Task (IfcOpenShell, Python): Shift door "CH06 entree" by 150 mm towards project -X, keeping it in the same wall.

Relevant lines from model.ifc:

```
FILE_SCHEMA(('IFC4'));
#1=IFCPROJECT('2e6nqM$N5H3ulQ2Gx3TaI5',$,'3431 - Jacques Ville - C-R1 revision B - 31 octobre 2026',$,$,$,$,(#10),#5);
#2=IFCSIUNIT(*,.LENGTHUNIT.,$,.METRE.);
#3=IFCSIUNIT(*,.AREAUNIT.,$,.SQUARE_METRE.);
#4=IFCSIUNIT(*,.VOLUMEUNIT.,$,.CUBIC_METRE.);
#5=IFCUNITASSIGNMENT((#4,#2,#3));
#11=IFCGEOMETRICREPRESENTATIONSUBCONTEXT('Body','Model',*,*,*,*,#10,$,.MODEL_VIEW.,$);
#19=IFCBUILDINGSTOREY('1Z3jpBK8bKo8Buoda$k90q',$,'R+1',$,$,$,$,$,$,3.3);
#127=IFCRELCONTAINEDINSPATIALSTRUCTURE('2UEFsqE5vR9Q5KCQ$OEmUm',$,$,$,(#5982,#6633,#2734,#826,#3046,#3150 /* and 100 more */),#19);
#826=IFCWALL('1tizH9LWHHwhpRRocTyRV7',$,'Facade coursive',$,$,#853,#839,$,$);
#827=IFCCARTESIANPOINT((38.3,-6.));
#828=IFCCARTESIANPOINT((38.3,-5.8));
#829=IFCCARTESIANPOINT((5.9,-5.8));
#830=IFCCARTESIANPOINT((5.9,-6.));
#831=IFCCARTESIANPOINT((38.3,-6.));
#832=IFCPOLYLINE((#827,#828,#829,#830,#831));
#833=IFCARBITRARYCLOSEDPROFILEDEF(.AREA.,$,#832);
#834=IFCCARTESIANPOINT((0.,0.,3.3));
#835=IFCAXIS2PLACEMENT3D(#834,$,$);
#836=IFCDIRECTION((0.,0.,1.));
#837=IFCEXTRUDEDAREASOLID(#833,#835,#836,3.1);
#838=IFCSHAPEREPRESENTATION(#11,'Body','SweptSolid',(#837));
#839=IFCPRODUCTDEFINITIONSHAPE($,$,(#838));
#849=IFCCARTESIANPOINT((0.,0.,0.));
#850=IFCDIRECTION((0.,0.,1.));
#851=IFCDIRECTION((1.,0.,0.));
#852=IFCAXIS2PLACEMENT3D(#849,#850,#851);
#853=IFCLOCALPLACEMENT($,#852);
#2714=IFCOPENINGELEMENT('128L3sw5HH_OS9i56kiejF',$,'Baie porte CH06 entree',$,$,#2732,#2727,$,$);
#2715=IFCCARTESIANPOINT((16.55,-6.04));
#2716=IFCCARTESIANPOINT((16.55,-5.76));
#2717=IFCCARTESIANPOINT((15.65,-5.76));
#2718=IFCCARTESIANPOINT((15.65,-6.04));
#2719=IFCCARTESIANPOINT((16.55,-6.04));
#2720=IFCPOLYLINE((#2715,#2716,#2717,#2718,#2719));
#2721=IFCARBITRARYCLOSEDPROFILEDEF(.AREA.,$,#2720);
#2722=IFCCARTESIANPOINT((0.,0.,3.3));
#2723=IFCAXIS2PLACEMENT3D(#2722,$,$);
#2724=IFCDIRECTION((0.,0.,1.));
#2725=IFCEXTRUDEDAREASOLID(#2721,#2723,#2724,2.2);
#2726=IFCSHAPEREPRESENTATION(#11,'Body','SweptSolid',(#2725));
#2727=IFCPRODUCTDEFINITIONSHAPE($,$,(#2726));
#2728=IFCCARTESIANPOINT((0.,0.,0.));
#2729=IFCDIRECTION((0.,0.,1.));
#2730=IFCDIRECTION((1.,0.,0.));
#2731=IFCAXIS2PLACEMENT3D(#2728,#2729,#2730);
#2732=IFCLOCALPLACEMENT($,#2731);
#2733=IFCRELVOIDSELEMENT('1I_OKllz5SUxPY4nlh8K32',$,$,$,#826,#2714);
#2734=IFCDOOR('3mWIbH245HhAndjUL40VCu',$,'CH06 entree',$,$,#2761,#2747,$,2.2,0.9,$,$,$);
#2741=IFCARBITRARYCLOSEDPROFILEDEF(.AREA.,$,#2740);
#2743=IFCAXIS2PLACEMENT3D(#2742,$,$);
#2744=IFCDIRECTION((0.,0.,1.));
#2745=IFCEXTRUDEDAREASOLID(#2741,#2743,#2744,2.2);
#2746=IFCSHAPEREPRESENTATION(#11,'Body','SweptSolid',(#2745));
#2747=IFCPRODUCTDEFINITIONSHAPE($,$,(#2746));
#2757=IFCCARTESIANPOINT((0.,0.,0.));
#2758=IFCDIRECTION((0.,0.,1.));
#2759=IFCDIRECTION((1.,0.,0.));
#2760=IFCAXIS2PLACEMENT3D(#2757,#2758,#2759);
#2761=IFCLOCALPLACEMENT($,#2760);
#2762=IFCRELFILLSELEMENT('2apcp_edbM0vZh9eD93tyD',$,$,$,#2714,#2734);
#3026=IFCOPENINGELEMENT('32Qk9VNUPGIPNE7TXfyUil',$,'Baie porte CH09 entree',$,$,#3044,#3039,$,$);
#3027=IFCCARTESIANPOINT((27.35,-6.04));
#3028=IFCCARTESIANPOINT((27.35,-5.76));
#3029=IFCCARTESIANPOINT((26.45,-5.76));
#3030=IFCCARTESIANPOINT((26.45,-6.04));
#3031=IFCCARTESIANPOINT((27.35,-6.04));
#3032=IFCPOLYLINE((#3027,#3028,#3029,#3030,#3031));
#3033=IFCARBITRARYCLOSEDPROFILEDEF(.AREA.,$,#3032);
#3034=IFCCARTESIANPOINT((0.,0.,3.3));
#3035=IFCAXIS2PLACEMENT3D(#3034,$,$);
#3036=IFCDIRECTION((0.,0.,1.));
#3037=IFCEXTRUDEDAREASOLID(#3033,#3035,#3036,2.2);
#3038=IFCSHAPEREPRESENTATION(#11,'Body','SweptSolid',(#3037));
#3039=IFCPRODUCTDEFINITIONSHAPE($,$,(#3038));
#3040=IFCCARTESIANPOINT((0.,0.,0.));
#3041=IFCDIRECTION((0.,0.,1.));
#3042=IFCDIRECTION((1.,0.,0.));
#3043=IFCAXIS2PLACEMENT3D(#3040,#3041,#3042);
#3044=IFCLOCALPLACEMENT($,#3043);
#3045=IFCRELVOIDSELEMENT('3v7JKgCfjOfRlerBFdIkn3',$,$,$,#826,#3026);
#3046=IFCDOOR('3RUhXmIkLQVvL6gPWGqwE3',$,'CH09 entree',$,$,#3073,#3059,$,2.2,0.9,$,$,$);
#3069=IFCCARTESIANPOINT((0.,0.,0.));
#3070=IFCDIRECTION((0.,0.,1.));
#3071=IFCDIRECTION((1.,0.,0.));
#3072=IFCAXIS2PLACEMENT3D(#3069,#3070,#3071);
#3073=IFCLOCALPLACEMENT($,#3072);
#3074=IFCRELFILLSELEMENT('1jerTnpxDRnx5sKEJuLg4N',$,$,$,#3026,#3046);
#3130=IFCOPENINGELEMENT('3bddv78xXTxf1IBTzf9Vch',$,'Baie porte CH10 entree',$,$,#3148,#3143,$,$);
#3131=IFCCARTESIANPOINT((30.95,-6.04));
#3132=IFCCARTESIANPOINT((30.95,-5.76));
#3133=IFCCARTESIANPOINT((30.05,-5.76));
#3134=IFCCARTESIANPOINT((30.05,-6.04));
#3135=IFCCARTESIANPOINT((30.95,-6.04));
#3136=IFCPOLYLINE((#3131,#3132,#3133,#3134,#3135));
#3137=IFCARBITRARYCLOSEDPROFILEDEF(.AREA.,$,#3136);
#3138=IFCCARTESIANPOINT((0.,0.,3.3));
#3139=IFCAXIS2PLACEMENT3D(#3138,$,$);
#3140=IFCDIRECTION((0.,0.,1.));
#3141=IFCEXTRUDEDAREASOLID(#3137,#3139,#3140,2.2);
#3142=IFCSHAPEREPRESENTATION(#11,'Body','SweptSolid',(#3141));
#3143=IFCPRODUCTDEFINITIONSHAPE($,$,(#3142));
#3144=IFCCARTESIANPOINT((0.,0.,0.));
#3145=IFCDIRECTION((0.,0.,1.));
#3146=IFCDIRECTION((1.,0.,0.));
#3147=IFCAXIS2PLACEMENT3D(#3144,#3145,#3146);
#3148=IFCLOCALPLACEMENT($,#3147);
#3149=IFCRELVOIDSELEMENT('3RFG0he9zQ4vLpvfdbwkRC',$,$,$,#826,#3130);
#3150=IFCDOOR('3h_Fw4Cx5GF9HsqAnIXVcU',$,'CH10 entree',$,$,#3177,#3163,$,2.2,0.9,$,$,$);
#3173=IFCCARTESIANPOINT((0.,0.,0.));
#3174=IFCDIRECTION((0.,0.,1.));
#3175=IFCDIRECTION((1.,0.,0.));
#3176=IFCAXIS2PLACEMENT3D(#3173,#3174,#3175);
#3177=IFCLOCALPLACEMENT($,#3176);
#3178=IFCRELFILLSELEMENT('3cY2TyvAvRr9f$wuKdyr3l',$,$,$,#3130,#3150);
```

```python
import ifcopenshell
import ifcopenshell.api.geometry
import ifcopenshell.util.placement
import ifcopenshell.util.unit

model = ifcopenshell.open("model.ifc")
unit_scale = ifcopenshell.util.unit.calculate_unit_scale(model)

door = model.by_guid("3mWIbH245HhAndjUL40VCu")
opening = door.FillsVoids[0].RelatingOpeningElement
wall = opening.VoidsElements[0].RelatingBuildingElement

wall_matrix = ifcopenshell.util.placement.get_local_placement(wall.ObjectPlacement)
shift = wall_matrix[:3, 0] * -0.15 / unit_scale
before = ifcopenshell.util.placement.get_local_placement(door.ObjectPlacement)[:3, 3].copy()

# The door is not placed relative to its opening, so move both.
for product in (opening, door):
    matrix = ifcopenshell.util.placement.get_local_placement(product.ObjectPlacement)
    matrix[:3, 3] += shift
    ifcopenshell.api.geometry.edit_object_placement(model, product=product, matrix=matrix, is_si=False)

after = ifcopenshell.util.placement.get_local_placement(door.ObjectPlacement)[:3, 3]
print("door moved by", (after - before).round(3) + 0.0)

model.write("model_rev.ifc")
```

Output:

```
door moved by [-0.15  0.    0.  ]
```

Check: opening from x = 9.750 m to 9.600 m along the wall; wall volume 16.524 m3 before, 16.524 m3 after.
